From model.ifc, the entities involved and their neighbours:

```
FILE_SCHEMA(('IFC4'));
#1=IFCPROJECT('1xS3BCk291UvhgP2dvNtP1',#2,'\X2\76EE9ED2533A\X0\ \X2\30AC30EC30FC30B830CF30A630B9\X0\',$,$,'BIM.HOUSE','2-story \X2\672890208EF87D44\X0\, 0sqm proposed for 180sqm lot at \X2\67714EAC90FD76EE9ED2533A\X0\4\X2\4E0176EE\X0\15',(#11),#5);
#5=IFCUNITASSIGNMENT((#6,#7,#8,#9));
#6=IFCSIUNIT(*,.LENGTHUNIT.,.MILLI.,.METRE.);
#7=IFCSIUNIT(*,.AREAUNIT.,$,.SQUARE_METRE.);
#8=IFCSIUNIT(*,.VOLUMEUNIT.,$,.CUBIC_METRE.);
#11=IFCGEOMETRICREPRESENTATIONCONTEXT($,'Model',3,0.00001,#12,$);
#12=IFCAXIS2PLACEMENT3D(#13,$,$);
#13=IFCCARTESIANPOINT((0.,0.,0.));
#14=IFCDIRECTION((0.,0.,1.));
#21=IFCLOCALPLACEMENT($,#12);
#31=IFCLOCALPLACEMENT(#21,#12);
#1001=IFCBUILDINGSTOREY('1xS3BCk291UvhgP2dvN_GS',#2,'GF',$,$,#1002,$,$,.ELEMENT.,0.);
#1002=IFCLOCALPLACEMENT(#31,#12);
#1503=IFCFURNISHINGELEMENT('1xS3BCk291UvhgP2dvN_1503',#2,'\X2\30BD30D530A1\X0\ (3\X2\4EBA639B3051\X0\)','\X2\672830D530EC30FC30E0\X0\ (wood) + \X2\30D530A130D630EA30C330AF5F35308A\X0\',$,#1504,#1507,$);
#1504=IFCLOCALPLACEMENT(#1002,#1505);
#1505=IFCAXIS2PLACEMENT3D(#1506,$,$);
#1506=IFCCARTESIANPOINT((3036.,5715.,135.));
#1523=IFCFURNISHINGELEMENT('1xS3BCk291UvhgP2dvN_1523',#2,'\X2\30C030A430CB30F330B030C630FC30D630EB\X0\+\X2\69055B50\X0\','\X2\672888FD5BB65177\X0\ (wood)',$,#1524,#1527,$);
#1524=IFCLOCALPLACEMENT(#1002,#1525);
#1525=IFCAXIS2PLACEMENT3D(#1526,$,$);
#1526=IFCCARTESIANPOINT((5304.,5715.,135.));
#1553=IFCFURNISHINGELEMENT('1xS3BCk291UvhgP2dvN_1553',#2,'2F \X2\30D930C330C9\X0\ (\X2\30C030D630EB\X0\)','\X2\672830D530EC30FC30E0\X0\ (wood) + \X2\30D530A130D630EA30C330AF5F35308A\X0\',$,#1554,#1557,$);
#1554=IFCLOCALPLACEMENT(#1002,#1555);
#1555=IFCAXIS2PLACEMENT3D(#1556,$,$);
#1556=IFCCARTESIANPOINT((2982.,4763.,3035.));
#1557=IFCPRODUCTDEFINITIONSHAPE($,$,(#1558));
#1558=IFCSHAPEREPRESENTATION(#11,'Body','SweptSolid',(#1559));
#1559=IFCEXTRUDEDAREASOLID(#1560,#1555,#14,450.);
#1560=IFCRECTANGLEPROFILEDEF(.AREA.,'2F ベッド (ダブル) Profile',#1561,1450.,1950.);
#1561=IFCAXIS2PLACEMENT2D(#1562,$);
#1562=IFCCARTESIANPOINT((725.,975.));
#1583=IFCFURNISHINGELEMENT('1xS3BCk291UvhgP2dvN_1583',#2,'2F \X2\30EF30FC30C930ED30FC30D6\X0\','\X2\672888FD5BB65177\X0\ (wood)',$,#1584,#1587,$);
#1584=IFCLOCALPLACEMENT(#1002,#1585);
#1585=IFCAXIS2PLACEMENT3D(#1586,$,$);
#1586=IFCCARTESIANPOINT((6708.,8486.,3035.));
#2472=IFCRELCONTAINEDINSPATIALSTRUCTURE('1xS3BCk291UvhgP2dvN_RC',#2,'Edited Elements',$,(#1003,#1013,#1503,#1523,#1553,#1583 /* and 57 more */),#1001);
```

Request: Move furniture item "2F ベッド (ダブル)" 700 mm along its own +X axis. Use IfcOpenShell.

```python
import ifcopenshell
import ifcopenshell.api.geometry
import ifcopenshell.util.placement
import ifcopenshell.util.unit

model = ifcopenshell.open("model.ifc")
unit_scale = ifcopenshell.util.unit.calculate_unit_scale(model)

item = model.by_guid("1xS3BCk291UvhgP2dvN_1553")
matrix = ifcopenshell.util.placement.get_local_placement(item.ObjectPlacement)
matrix[:3, 3] += matrix[:3, 0] * 0.7 / unit_scale
ifcopenshell.api.geometry.edit_object_placement(model, product=item, matrix=matrix, is_si=False)

print(ifcopenshell.util.placement.get_local_placement(item.ObjectPlacement).round(3) + 0.0)

model.write("model-out.ifc")
```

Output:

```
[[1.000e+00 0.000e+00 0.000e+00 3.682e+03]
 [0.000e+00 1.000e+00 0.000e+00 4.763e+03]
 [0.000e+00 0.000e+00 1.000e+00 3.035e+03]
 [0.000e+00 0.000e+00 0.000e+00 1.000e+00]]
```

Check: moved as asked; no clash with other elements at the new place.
